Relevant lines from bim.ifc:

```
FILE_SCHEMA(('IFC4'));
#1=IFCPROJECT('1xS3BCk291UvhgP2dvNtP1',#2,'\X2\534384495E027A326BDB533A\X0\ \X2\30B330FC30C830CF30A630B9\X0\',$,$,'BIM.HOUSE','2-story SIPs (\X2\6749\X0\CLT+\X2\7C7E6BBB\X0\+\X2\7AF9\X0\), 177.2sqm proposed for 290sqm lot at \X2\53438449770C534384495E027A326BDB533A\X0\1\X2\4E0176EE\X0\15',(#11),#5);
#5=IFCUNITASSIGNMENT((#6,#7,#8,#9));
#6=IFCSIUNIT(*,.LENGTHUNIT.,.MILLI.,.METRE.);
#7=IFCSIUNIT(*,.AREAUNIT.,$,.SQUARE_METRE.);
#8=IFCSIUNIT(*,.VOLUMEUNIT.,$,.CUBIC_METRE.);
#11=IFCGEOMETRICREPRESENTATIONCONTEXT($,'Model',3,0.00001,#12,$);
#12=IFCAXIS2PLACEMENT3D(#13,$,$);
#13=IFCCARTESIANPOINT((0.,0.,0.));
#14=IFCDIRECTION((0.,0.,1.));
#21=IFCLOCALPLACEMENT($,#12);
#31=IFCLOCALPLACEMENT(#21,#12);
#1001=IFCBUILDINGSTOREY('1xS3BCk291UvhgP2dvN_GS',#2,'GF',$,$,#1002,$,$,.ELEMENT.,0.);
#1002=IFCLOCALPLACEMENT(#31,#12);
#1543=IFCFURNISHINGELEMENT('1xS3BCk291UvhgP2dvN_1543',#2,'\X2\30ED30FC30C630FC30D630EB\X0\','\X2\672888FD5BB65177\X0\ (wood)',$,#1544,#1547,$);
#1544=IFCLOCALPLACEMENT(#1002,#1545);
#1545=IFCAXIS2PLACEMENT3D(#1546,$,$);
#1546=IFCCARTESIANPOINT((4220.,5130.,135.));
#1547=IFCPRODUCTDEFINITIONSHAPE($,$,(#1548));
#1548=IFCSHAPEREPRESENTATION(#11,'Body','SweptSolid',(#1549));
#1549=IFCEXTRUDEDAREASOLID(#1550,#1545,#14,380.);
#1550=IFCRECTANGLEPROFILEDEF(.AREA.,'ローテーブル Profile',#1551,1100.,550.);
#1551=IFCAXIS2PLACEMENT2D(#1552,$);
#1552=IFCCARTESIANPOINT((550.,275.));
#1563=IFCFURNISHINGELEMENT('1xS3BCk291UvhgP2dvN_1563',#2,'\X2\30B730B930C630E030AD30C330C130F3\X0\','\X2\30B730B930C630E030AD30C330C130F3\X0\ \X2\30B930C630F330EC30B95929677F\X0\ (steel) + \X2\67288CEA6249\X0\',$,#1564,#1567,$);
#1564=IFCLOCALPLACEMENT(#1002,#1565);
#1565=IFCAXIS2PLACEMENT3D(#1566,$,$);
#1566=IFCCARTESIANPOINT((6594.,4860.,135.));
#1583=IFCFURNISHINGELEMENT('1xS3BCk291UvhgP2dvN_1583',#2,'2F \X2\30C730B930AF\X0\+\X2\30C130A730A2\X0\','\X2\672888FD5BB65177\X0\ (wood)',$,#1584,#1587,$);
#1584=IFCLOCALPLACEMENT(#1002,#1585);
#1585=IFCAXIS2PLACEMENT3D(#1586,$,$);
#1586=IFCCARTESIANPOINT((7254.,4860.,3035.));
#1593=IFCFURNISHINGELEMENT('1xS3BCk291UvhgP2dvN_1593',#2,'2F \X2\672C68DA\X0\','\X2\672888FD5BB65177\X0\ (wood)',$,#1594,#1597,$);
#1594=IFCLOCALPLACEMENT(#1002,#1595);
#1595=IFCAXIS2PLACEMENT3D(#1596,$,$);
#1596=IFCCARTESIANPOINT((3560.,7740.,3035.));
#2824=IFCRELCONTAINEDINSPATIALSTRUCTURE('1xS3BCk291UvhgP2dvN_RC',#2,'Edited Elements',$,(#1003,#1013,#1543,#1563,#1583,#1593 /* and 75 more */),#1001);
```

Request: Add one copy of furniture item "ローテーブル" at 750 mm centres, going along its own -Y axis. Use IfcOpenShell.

```python
import ifcopenshell
import ifcopenshell.api.geometry
import ifcopenshell.api.root
import ifcopenshell.util.element
import ifcopenshell.util.placement

model = ifcopenshell.open("bim.ifc")


def reuse_history(source, copy):
    """copy_class also copies each property set's owner history, people and application; keep the originals."""
    for rel in copy.IsDefinedBy:
        if rel.is_a("IfcRelDefinesByProperties") and (history := rel.RelatingPropertyDefinition.OwnerHistory):
            rel.RelatingPropertyDefinition.OwnerHistory = source.OwnerHistory
            ifcopenshell.util.element.remove_deep2(model, history)


source = model.by_guid("1xS3BCk291UvhgP2dvN_1543")
base = ifcopenshell.util.placement.get_local_placement(source.ObjectPlacement)
step = -base[:3, 1] * 750.0

for i in range(1, 2):
    copy = ifcopenshell.api.root.copy_class(model, product=source)
    copy.Representation = ifcopenshell.util.element.copy_deep(
        model, source.Representation, exclude=["IfcGeometricRepresentationContext", "IfcRepresentationMap"]
    )
    reuse_history(source, copy)
    matrix = base.copy()
    matrix[:3, 3] += i * step
    print("added at", matrix[:3, 3].round(3) + 0.0)
    ifcopenshell.api.geometry.edit_object_placement(model, product=copy, matrix=matrix, is_si=False)

model.write("bim_updated.ifc")
```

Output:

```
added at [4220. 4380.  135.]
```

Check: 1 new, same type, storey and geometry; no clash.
